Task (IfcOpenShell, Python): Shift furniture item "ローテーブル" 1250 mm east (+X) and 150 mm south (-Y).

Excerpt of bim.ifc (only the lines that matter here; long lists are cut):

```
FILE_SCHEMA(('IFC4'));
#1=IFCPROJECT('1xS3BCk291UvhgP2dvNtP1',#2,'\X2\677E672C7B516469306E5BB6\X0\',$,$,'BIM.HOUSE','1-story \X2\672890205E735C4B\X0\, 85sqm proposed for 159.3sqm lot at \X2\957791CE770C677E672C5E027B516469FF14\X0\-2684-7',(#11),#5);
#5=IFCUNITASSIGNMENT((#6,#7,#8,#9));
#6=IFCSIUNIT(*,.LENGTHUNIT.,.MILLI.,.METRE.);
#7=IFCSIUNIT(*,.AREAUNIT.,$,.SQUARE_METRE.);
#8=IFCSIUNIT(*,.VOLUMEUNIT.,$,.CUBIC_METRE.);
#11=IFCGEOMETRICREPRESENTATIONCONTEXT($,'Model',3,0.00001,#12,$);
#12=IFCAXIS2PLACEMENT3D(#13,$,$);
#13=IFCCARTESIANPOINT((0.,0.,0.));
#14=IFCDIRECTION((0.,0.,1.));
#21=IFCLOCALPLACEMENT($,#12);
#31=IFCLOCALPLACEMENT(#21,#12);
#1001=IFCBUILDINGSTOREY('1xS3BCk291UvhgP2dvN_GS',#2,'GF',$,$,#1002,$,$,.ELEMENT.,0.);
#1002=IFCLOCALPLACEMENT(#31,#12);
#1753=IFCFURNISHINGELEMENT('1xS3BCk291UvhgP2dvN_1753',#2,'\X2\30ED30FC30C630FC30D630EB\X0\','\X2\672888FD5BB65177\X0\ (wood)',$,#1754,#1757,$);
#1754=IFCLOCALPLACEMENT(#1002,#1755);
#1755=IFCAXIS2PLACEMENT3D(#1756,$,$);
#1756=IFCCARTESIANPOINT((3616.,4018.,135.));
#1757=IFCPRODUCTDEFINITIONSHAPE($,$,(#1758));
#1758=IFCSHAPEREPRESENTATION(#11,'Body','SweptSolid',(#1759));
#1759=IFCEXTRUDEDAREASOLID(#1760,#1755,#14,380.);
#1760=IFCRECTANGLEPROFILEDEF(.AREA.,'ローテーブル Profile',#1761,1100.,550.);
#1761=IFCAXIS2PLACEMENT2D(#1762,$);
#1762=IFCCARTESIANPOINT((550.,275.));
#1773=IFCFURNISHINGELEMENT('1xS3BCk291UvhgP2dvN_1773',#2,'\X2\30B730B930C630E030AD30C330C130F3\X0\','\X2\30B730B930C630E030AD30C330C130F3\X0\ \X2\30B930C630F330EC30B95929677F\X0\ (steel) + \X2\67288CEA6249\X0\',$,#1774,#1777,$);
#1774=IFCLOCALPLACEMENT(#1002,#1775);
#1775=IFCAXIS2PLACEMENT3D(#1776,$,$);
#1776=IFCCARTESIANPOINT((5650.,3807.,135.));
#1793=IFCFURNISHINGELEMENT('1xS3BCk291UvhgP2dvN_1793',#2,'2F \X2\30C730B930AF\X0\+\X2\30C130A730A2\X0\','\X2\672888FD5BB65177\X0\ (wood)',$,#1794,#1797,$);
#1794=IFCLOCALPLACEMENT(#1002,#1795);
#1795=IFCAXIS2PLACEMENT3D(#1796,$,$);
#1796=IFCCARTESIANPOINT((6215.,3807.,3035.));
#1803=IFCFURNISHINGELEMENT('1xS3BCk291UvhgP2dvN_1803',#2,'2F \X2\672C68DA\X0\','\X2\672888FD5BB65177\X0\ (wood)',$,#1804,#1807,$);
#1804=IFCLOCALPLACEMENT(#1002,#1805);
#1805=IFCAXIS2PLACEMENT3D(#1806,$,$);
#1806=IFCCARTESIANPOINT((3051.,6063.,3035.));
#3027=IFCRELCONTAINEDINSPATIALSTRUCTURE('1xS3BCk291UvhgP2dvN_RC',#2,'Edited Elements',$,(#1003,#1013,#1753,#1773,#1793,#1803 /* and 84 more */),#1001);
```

```python
import ifcopenshell
import ifcopenshell.api.geometry
import ifcopenshell.util.placement
import ifcopenshell.util.unit

model = ifcopenshell.open("bim.ifc")
unit_scale = ifcopenshell.util.unit.calculate_unit_scale(model)

item = model.by_guid("1xS3BCk291UvhgP2dvN_1753")
matrix = ifcopenshell.util.placement.get_local_placement(item.ObjectPlacement)
matrix[0, 3] += 1.25 / unit_scale
matrix[1, 3] -= 0.15 / unit_scale
ifcopenshell.api.geometry.edit_object_placement(model, product=item, matrix=matrix, is_si=False)

print(ifcopenshell.util.placement.get_local_placement(item.ObjectPlacement).round(3) + 0.0)

model.write("bim_edited.ifc")
```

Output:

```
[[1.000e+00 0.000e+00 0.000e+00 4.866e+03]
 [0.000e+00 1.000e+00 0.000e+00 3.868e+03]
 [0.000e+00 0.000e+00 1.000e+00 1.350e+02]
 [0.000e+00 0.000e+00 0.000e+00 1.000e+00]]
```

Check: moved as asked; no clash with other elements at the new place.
